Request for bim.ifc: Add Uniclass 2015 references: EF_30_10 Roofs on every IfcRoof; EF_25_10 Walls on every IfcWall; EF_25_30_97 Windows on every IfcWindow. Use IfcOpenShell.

First a look at what the model holds.

```python
import ifcopenshell

model = ifcopenshell.open("bim.ifc")
print(model.schema)
print("classifications:", [c.Name for c in model.by_type("IfcClassification")])
for ifc_class in ("IfcDoor", "IfcRoof", "IfcStair", "IfcWall", "IfcWindow"):
    print(ifc_class, len(model.by_type(ifc_class)))
```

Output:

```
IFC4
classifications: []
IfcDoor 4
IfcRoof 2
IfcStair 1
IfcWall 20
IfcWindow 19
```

```python
import ifcopenshell
import ifcopenshell.api.classification

model = ifcopenshell.open("bim.ifc")

system = ifcopenshell.api.classification.add_classification(model, classification="Uniclass 2015")

codes = {
    "IfcRoof": ("EF_30_10", "Roofs"),
    "IfcWall": ("EF_25_10", "Walls"),
    "IfcWindow": ("EF_25_30_97", "Windows"),
}
for ifc_class, (code, name) in codes.items():
    products = model.by_type(ifc_class)
    ifcopenshell.api.classification.add_reference(
        model, products=products, classification=system, identification=code, name=name
    )
    print(code, len(products))

model.write("bim-out.ifc")
```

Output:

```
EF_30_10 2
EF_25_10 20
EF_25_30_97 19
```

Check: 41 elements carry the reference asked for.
